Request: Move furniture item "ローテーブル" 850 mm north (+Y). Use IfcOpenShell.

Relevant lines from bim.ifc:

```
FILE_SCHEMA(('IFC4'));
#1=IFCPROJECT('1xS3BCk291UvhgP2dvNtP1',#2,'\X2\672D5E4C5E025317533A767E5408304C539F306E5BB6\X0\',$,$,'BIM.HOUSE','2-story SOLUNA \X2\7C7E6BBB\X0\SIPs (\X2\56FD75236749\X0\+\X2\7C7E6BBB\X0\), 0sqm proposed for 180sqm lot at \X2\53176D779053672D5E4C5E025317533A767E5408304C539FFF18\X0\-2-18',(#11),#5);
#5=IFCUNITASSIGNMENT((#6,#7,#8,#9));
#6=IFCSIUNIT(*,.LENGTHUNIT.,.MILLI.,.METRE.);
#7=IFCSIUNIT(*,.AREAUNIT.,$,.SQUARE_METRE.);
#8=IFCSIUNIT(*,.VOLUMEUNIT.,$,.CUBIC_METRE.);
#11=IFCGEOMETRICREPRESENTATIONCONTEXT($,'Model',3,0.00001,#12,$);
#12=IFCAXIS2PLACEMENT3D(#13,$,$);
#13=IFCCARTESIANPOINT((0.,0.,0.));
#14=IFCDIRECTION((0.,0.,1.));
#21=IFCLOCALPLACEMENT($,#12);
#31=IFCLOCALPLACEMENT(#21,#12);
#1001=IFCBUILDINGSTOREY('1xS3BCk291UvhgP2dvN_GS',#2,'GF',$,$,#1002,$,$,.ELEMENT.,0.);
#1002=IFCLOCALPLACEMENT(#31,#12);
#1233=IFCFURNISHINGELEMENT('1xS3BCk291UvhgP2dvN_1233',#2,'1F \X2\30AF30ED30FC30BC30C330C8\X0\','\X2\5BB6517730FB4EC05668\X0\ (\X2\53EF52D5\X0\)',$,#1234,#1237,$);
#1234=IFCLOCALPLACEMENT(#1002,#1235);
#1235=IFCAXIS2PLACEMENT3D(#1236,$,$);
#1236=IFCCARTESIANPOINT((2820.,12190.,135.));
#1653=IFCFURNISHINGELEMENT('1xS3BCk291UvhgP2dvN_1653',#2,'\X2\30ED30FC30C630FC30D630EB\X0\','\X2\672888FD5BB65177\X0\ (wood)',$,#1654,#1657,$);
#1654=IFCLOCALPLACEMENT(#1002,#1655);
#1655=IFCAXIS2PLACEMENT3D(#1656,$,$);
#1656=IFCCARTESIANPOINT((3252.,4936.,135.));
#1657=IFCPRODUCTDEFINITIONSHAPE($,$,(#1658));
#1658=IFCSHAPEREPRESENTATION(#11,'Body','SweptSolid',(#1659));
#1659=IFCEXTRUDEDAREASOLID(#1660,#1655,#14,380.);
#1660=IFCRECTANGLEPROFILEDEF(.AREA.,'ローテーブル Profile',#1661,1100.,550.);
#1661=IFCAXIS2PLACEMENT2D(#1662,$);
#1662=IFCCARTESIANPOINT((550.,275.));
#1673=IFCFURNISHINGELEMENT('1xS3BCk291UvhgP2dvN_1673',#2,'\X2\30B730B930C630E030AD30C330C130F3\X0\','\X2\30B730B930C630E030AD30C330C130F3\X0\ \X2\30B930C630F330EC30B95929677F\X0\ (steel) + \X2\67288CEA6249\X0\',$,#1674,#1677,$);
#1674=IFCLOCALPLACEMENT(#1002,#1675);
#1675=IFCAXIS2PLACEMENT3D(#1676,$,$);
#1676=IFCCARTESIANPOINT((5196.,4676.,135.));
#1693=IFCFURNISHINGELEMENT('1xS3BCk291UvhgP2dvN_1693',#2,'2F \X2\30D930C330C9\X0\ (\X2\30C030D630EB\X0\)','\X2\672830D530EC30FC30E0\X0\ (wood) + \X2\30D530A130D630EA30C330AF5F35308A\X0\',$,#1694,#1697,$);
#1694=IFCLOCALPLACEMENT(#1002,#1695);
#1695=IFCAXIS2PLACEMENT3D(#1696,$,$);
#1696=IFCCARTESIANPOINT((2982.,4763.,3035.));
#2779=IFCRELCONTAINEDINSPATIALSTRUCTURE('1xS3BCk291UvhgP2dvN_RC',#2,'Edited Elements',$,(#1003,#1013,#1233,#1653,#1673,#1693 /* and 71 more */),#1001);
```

```python
import ifcopenshell
import ifcopenshell.api.geometry
import ifcopenshell.util.placement
import ifcopenshell.util.unit

model = ifcopenshell.open("bim.ifc")
unit_scale = ifcopenshell.util.unit.calculate_unit_scale(model)

item = model.by_guid("1xS3BCk291UvhgP2dvN_1653")
matrix = ifcopenshell.util.placement.get_local_placement(item.ObjectPlacement)
matrix[1, 3] += 0.85 / unit_scale
ifcopenshell.api.geometry.edit_object_placement(model, product=item, matrix=matrix, is_si=False)

print(ifcopenshell.util.placement.get_local_placement(item.ObjectPlacement).round(3) + 0.0)

model.write("bim_rev.ifc")
```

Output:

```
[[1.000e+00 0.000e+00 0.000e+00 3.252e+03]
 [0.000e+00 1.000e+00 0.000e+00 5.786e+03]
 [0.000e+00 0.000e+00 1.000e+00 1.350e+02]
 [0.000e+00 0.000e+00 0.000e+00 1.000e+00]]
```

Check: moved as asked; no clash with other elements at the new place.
